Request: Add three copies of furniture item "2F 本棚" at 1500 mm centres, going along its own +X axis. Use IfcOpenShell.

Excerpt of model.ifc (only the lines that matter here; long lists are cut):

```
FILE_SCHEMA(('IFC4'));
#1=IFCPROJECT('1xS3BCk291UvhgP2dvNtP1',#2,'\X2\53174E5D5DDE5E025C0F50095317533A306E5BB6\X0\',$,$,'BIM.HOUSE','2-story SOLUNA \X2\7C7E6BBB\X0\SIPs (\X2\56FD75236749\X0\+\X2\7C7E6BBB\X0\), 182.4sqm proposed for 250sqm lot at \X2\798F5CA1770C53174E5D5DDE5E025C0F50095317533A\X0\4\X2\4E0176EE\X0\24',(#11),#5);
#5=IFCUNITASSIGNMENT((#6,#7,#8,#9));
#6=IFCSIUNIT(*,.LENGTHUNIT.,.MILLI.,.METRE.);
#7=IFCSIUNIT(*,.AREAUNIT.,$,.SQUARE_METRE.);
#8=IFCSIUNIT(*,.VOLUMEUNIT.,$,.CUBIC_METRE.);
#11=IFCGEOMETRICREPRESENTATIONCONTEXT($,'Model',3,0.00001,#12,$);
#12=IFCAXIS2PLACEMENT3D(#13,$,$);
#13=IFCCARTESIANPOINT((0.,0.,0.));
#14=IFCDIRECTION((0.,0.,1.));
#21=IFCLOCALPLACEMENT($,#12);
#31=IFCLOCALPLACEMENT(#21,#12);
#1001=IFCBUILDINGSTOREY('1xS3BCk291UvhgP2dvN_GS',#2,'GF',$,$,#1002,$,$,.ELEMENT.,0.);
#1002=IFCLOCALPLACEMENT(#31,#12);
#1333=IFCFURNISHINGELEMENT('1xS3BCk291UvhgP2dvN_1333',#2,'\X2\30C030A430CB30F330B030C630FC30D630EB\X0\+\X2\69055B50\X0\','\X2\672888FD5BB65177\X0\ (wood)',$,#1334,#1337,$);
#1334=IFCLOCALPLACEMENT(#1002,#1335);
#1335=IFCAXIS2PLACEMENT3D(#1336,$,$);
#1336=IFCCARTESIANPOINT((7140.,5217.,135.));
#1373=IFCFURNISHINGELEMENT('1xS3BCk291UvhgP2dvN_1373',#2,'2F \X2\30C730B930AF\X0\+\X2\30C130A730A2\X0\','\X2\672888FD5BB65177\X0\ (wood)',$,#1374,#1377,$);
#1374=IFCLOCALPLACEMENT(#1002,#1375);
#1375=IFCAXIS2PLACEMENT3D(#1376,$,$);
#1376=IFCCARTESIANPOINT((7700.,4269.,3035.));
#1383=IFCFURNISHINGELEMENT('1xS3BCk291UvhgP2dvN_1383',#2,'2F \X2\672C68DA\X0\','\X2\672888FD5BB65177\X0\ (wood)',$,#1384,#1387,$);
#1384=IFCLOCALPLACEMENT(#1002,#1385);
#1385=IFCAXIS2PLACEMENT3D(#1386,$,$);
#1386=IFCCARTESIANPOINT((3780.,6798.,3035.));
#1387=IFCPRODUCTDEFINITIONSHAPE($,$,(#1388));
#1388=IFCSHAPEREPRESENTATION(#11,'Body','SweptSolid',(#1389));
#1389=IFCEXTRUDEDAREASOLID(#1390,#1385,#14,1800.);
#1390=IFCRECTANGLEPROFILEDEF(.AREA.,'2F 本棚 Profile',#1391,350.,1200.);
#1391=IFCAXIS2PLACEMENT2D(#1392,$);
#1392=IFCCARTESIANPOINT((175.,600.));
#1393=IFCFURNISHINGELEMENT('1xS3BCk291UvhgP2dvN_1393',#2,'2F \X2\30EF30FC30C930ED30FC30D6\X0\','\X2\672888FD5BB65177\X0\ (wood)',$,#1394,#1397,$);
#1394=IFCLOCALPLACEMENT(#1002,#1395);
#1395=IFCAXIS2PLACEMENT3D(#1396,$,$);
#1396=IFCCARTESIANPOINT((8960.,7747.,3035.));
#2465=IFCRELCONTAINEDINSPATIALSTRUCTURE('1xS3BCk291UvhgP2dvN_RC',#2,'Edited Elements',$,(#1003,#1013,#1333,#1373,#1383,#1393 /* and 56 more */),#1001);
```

```python
import ifcopenshell
import ifcopenshell.api.geometry
import ifcopenshell.api.root
import ifcopenshell.util.element
import ifcopenshell.util.placement
import ifcopenshell.util.unit

model = ifcopenshell.open("model.ifc")
unit_scale = ifcopenshell.util.unit.calculate_unit_scale(model)


def reuse_history(source, copy):
    """copy_class also copies each property set's owner history, people and application; keep the originals."""
    for rel in copy.IsDefinedBy:
        if rel.is_a("IfcRelDefinesByProperties") and (history := rel.RelatingPropertyDefinition.OwnerHistory):
            rel.RelatingPropertyDefinition.OwnerHistory = source.OwnerHistory
            ifcopenshell.util.element.remove_deep2(model, history)


source = model.by_guid("1xS3BCk291UvhgP2dvN_1383")
base = ifcopenshell.util.placement.get_local_placement(source.ObjectPlacement)
step = base[:3, 0] * 1.5 / unit_scale

for i in range(1, 4):
    copy = ifcopenshell.api.root.copy_class(model, product=source)
    copy.Representation = ifcopenshell.util.element.copy_deep(
        model, source.Representation, exclude=["IfcGeometricRepresentationContext", "IfcRepresentationMap"]
    )
    reuse_history(source, copy)
    matrix = base.copy()
    matrix[:3, 3] += i * step
    print("added at", matrix[:3, 3].round(3) + 0.0)
    ifcopenshell.api.geometry.edit_object_placement(model, product=copy, matrix=matrix, is_si=False)

model.write("model_rev.ifc")
```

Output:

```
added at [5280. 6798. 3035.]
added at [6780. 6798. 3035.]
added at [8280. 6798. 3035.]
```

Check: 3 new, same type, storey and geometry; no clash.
